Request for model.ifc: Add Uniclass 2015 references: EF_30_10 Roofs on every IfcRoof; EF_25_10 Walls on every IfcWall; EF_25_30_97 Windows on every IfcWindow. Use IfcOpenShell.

First a look at what the model holds.

```python
import ifcopenshell

model = ifcopenshell.open("model.ifc")
print(model.schema)
print("classifications:", [c.Name for c in model.by_type("IfcClassification")])
for ifc_class in ("IfcDoor", "IfcRoof", "IfcStair", "IfcWall", "IfcWindow"):
    print(ifc_class, len(model.by_type(ifc_class)))
```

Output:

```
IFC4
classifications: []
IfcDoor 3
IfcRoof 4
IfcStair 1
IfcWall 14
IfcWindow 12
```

```python
import ifcopenshell
import ifcopenshell.api.classification

model = ifcopenshell.open("model.ifc")

system = ifcopenshell.api.classification.add_classification(model, classification="Uniclass 2015")

codes = {
    "IfcRoof": ("EF_30_10", "Roofs"),
    "IfcWall": ("EF_25_10", "Walls"),
    "IfcWindow": ("EF_25_30_97", "Windows"),
}
for ifc_class, (code, name) in codes.items():
    products = model.by_type(ifc_class)
    ifcopenshell.api.classification.add_reference(
        model, products=products, classification=system, identification=code, name=name
    )
    print(code, len(products))

model.write("model-out.ifc")
```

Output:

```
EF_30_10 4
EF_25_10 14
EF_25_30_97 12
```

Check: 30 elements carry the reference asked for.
